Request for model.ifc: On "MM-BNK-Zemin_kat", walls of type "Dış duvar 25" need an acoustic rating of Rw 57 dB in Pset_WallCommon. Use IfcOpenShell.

First a look at what the model holds.

```python
import ifcopenshell
import ifcopenshell.util.element

model = ifcopenshell.open("model.ifc")
print(model.schema)
storey = next(s for s in model.by_type("IfcBuildingStorey") if s.Name == "MM-BNK-Zemin_kat")
walls = [e for e in ifcopenshell.util.element.get_decomposition(storey) if e.is_a("IfcWall")]
seen = {}
for e in walls:
    element_type = ifcopenshell.util.element.get_type(e)
    key = (element_type.Name if element_type != e and element_type else None, ifcopenshell.util.element.get_pset(e, "Pset_WallCommon", "AcousticRating"))
    seen[key] = seen.get(key, 0) + 1
for (name, value), count in sorted(seen.items(), key=str):
    print(count, "x", name, "|", value)
```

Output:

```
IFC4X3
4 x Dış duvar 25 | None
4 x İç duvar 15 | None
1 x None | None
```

```python
import ifcopenshell
import ifcopenshell.api.pset
import ifcopenshell.util.element

model = ifcopenshell.open("model.ifc")

storey = next(s for s in model.by_type("IfcBuildingStorey") if s.Name == "MM-BNK-Zemin_kat")
walls = [e for e in ifcopenshell.util.element.get_decomposition(storey) if e.is_a("IfcWall")]

count = 0
for e in walls:
    element_type = ifcopenshell.util.element.get_type(e)
    if element_type in (None, e) or element_type.Name != "Dış duvar 25":
        continue
    # add_pset returns the element's existing set when there is one.
    pset = ifcopenshell.api.pset.add_pset(model, product=e, name="Pset_WallCommon")
    ifcopenshell.api.pset.edit_pset(model, pset=pset, properties={"AcousticRating": "Rw 57 dB"})
    count += 1

print(count, "walls updated")

model.write("model-out.ifc")
```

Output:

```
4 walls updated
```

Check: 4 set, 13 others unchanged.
